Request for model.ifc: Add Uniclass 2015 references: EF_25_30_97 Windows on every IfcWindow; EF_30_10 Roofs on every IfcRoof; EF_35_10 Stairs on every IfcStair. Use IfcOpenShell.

First a look at what the model holds.

```python
import ifcopenshell

model = ifcopenshell.open("model.ifc")
print(model.schema)
print("classifications:", [c.Name for c in model.by_type("IfcClassification")])
for ifc_class in ("IfcDoor", "IfcRoof", "IfcStair", "IfcWall", "IfcWindow"):
    print(ifc_class, len(model.by_type(ifc_class)))
```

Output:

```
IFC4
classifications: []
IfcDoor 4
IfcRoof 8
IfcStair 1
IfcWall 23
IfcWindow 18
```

```python
import ifcopenshell
import ifcopenshell.api.classification

model = ifcopenshell.open("model.ifc")

system = ifcopenshell.api.classification.add_classification(model, classification="Uniclass 2015")

codes = {
    "IfcWindow": ("EF_25_30_97", "Windows"),
    "IfcRoof": ("EF_30_10", "Roofs"),
    "IfcStair": ("EF_35_10", "Stairs"),
}
for ifc_class, (code, name) in codes.items():
    products = model.by_type(ifc_class)
    ifcopenshell.api.classification.add_reference(
        model, products=products, classification=system, identification=code, name=name
    )
    print(code, len(products))

model.write("model-out.ifc")
```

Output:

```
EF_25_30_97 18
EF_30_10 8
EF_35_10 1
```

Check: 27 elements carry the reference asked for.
